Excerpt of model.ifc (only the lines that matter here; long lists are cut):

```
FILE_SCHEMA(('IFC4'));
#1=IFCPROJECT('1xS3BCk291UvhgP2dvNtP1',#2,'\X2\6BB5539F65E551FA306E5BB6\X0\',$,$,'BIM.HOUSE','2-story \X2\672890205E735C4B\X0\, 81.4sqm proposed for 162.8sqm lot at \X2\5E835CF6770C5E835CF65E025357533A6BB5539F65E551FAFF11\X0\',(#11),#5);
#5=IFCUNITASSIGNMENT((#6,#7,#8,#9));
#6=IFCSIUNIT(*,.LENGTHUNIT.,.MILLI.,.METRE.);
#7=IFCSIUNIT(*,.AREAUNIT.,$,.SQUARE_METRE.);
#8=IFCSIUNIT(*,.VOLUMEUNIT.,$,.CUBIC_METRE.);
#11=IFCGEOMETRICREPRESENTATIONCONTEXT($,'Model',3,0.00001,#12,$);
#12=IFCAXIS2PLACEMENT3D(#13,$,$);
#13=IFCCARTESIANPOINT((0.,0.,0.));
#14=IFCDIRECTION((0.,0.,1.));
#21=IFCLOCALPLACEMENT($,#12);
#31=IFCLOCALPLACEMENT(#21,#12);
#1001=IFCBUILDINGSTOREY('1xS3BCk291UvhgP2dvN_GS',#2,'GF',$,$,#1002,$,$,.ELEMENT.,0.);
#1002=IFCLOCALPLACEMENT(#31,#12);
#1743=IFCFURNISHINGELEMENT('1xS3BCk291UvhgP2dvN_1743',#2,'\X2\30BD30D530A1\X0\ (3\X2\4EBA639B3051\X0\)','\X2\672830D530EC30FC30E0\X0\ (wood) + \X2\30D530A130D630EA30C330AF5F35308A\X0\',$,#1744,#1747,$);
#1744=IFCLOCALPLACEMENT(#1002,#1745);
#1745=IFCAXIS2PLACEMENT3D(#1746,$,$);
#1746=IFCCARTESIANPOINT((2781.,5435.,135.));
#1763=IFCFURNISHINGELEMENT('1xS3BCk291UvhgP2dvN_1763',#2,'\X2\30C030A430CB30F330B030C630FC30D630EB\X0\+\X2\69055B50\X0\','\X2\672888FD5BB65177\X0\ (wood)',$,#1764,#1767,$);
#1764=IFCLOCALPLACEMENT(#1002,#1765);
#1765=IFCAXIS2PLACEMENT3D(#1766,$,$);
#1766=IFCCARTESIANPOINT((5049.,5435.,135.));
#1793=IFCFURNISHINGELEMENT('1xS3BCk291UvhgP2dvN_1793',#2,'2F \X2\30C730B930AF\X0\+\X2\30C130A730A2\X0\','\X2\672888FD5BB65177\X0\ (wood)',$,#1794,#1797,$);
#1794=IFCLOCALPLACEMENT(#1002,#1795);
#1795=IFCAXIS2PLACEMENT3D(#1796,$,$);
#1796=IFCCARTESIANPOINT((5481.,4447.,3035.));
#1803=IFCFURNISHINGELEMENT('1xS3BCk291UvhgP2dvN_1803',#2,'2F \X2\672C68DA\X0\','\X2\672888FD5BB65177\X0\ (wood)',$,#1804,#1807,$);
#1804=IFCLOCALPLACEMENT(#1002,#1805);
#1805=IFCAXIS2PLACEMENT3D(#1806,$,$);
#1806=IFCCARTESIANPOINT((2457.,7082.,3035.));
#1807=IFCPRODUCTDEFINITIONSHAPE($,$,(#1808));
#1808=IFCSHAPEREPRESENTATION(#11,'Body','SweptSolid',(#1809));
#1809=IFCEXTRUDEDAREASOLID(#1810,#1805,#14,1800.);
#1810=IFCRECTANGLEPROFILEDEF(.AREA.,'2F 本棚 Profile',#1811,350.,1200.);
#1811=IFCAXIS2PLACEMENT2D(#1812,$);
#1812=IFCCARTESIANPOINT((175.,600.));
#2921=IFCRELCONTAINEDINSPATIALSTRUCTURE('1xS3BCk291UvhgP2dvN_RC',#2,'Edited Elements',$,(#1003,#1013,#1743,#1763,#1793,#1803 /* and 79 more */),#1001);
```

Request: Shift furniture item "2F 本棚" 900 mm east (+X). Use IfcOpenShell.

```python
import ifcopenshell
import ifcopenshell.api.geometry
import ifcopenshell.util.placement

model = ifcopenshell.open("model.ifc")

item = model.by_guid("1xS3BCk291UvhgP2dvN_1803")
matrix = ifcopenshell.util.placement.get_local_placement(item.ObjectPlacement)
matrix[0, 3] += 900.0
ifcopenshell.api.geometry.edit_object_placement(model, product=item, matrix=matrix, is_si=False)

print(ifcopenshell.util.placement.get_local_placement(item.ObjectPlacement).round(3) + 0.0)

model.write("model-out.ifc")
```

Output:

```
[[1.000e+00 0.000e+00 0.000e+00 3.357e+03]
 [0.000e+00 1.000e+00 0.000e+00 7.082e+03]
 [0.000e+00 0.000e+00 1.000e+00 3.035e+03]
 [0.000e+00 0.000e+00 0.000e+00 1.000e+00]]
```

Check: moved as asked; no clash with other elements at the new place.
